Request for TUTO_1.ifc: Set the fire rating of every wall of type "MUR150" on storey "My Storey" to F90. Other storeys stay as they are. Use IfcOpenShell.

First a look at what the model holds.

```python
import ifcopenshell
import ifcopenshell.util.element

model = ifcopenshell.open("TUTO_1.ifc")
print(model.schema)
storey = next(s for s in model.by_type("IfcBuildingStorey") if s.Name == "My Storey")
walls = [e for e in ifcopenshell.util.element.get_decomposition(storey) if e.is_a("IfcWall")]
seen = {}
for e in walls:
    element_type = ifcopenshell.util.element.get_type(e)
    key = (element_type.Name if element_type != e and element_type else None, ifcopenshell.util.element.get_pset(e, "Pset_WallCommon", "FireRating"))
    seen[key] = seen.get(key, 0) + 1
for (name, value), count in sorted(seen.items(), key=str):
    print(count, "x", name, "|", value)
```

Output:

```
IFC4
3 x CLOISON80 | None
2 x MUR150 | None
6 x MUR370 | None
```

```python
import ifcopenshell
import ifcopenshell.api.pset
import ifcopenshell.util.element

model = ifcopenshell.open("TUTO_1.ifc")

storey = next(s for s in model.by_type("IfcBuildingStorey") if s.Name == "My Storey")
walls = [e for e in ifcopenshell.util.element.get_decomposition(storey) if e.is_a("IfcWall")]

count = 0
for e in walls:
    element_type = ifcopenshell.util.element.get_type(e)
    if element_type in (None, e) or element_type.Name != "MUR150":
        continue
    # add_pset returns the element's existing set when there is one.
    pset = ifcopenshell.api.pset.add_pset(model, product=e, name="Pset_WallCommon")
    ifcopenshell.api.pset.edit_pset(model, pset=pset, properties={"FireRating": "F90"})
    count += 1

print(count, "walls updated")

model.write("TUTO_1_updated.ifc")
```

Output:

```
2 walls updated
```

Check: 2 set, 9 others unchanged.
